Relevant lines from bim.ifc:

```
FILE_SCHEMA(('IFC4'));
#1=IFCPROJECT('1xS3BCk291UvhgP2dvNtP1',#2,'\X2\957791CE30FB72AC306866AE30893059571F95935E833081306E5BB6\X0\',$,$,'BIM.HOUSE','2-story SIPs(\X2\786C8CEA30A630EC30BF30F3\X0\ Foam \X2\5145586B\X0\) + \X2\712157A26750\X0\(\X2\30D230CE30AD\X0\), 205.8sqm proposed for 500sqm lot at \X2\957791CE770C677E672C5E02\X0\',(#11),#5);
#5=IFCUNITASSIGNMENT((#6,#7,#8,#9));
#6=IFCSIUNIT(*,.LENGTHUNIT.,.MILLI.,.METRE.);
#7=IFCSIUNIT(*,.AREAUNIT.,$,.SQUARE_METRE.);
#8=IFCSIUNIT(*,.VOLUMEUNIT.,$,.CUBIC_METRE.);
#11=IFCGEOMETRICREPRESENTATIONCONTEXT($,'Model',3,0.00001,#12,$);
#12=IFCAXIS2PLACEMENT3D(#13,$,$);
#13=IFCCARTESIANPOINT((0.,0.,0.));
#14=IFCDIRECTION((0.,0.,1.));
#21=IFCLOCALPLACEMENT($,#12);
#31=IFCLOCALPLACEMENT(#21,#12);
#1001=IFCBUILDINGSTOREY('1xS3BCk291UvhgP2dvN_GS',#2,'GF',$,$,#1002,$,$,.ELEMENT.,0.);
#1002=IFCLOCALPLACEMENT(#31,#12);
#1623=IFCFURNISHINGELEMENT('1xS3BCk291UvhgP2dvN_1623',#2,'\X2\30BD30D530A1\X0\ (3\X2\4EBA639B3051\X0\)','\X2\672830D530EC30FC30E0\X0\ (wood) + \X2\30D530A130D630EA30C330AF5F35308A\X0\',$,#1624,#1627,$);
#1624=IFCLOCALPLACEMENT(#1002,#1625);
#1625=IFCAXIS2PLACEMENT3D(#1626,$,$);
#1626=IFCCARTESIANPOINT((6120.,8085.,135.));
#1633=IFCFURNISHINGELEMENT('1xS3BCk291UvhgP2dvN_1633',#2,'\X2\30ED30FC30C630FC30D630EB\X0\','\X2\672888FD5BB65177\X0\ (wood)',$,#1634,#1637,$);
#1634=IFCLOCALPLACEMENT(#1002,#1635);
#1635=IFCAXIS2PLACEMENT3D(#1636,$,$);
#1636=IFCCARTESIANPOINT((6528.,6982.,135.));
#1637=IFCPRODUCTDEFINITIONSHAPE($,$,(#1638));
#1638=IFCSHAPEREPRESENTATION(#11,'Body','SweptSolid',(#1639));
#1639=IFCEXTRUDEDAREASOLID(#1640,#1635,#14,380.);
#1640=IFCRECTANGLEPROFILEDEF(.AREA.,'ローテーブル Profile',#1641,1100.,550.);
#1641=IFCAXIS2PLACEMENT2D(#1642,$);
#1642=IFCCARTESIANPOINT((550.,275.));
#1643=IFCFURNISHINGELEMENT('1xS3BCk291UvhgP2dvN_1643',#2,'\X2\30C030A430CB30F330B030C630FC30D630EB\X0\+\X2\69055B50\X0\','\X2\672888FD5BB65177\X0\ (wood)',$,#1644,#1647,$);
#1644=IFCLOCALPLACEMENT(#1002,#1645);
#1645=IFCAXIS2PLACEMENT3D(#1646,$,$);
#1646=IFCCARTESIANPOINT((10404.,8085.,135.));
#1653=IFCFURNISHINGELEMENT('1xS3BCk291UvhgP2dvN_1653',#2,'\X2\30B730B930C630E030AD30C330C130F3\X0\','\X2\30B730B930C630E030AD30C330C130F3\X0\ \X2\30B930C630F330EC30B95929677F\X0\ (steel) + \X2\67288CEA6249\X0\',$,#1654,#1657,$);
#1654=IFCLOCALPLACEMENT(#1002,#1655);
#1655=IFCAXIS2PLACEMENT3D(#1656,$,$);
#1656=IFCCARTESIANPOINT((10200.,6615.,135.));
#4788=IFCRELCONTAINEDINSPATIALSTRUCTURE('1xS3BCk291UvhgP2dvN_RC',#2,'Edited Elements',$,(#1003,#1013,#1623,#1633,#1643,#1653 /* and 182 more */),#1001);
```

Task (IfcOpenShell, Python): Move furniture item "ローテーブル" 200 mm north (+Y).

```python
import ifcopenshell
import ifcopenshell.api.geometry
import ifcopenshell.util.placement
import ifcopenshell.util.unit

model = ifcopenshell.open("bim.ifc")
unit_scale = ifcopenshell.util.unit.calculate_unit_scale(model)

item = model.by_guid("1xS3BCk291UvhgP2dvN_1633")
matrix = ifcopenshell.util.placement.get_local_placement(item.ObjectPlacement)
matrix[1, 3] += 0.2 / unit_scale
ifcopenshell.api.geometry.edit_object_placement(model, product=item, matrix=matrix, is_si=False)

print(ifcopenshell.util.placement.get_local_placement(item.ObjectPlacement).round(3) + 0.0)

model.write("bim_rev.ifc")
```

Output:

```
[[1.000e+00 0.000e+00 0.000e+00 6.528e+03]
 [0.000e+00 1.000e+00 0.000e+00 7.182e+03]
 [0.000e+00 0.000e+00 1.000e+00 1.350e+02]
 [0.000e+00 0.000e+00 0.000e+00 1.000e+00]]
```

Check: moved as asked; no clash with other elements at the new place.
